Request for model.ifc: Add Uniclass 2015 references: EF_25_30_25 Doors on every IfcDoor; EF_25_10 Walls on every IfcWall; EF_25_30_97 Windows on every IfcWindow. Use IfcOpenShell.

First a look at what the model holds.

```python
import ifcopenshell

model = ifcopenshell.open("model.ifc")
print(model.schema)
print("classifications:", [c.Name for c in model.by_type("IfcClassification")])
for ifc_class in ("IfcDoor", "IfcRoof", "IfcStair", "IfcWall", "IfcWindow"):
    print(ifc_class, len(model.by_type(ifc_class)))
```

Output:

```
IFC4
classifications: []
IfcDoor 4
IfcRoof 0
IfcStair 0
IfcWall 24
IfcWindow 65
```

```python
import ifcopenshell
import ifcopenshell.api.classification

model = ifcopenshell.open("model.ifc")

system = ifcopenshell.api.classification.add_classification(model, classification="Uniclass 2015")

codes = {
    "IfcDoor": ("EF_25_30_25", "Doors"),
    "IfcWall": ("EF_25_10", "Walls"),
    "IfcWindow": ("EF_25_30_97", "Windows"),
}
for ifc_class, (code, name) in codes.items():
    products = model.by_type(ifc_class)
    ifcopenshell.api.classification.add_reference(
        model, products=products, classification=system, identification=code, name=name
    )
    print(code, len(products))

model.write("model_updated.ifc")
```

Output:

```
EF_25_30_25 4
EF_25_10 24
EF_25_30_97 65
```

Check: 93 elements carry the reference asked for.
